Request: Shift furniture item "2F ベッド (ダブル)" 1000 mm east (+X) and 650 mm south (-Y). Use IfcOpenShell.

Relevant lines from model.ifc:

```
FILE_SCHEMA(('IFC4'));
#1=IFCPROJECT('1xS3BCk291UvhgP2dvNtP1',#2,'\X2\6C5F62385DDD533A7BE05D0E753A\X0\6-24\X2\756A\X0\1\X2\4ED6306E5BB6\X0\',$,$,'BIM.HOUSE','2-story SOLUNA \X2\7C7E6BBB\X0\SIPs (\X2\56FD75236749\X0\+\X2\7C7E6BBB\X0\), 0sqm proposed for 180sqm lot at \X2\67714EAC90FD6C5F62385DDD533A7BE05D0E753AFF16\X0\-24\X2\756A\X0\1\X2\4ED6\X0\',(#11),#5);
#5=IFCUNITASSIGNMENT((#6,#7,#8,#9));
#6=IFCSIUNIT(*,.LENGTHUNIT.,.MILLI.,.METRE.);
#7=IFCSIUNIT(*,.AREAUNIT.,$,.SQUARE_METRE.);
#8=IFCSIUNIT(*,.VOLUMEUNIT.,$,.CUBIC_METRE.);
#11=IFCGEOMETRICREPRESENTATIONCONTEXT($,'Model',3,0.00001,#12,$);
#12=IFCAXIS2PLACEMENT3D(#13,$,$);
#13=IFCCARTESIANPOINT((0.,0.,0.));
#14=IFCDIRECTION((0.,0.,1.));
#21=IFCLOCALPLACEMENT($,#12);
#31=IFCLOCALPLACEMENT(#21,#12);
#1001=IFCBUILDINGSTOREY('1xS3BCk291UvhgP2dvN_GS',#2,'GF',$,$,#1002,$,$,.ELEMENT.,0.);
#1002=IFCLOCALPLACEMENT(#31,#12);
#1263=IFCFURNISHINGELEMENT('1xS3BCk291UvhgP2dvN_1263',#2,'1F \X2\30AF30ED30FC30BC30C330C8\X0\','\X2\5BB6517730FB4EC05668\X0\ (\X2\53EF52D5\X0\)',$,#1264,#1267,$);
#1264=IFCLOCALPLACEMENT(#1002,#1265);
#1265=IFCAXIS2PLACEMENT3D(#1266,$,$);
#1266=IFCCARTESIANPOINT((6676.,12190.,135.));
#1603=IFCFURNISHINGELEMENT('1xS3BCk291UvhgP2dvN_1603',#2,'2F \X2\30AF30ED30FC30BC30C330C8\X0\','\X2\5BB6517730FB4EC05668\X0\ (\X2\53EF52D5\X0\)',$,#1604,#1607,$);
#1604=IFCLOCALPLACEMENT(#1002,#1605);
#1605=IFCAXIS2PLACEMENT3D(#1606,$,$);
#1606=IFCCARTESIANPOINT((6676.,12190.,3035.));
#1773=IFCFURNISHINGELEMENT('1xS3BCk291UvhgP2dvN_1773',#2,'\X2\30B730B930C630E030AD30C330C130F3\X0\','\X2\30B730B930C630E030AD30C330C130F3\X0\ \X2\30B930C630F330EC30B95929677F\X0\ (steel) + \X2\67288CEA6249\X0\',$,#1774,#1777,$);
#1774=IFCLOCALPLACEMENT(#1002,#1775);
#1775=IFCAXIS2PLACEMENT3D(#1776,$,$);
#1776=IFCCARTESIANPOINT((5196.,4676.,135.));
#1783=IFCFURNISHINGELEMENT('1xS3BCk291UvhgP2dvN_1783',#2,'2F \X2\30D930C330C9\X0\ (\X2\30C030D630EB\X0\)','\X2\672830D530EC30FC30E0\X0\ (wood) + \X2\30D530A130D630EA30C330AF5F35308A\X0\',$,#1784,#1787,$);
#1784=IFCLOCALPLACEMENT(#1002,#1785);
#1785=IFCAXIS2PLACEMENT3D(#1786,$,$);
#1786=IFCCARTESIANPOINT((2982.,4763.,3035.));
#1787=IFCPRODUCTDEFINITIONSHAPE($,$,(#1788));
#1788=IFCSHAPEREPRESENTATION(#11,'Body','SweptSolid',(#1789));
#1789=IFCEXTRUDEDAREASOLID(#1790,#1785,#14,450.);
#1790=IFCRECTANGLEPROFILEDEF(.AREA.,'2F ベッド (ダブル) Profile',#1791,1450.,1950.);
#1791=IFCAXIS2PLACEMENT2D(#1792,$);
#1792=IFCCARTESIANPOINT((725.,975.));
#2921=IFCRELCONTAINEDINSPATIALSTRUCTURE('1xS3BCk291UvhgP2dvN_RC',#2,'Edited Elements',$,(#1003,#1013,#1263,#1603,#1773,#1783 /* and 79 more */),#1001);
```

```python
import ifcopenshell
import ifcopenshell.api.geometry
import ifcopenshell.util.placement
import ifcopenshell.util.unit

model = ifcopenshell.open("model.ifc")
unit_scale = ifcopenshell.util.unit.calculate_unit_scale(model)

item = model.by_guid("1xS3BCk291UvhgP2dvN_1783")
matrix = ifcopenshell.util.placement.get_local_placement(item.ObjectPlacement)
matrix[0, 3] += 1 / unit_scale
matrix[1, 3] -= 0.65 / unit_scale
ifcopenshell.api.geometry.edit_object_placement(model, product=item, matrix=matrix, is_si=False)

print(ifcopenshell.util.placement.get_local_placement(item.ObjectPlacement).round(3) + 0.0)

model.write("model_rev.ifc")
```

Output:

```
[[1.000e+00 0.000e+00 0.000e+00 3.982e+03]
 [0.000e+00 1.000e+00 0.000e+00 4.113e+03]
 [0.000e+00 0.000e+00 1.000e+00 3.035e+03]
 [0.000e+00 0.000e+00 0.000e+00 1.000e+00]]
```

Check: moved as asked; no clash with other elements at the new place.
